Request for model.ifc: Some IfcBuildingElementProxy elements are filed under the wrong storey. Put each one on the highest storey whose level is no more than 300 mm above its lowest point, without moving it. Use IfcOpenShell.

First a look at what the model holds.

```python
import ifcopenshell
import ifcopenshell.util.element
import ifcopenshell.util.placement

model = ifcopenshell.open("model.ifc")
print(model.schema)
for storey in model.by_type("IfcBuildingStorey"):
    level = ifcopenshell.util.placement.get_storey_elevation(storey)
    count = sum(e.is_a("IfcBuildingElementProxy") for e in ifcopenshell.util.element.get_contained(storey))
    print(storey.id(), storey.Name, round(level, 3), count, sep=" | ")
```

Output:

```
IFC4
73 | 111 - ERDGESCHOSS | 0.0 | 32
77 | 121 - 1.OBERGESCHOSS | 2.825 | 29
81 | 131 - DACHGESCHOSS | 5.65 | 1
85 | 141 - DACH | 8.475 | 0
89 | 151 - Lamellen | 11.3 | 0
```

```python
import ifcopenshell
import ifcopenshell.api.spatial
import ifcopenshell.geom
import ifcopenshell.util.element
import ifcopenshell.util.placement
import ifcopenshell.util.shape
import ifcopenshell.util.unit

model = ifcopenshell.open("model.ifc")
unit_scale = ifcopenshell.util.unit.calculate_unit_scale(model)
settings = ifcopenshell.geom.settings()

levels = sorted(
    ((ifcopenshell.util.placement.get_storey_elevation(s) * unit_scale, s) for s in model.by_type("IfcBuildingStorey")),
    key=lambda pair: pair[0],
)

for e in model.by_type("IfcBuildingElementProxy"):
    current = e.ContainedInStructure[0].RelatingStructure if e.ContainedInStructure else None
    if current is None or not current.is_a("IfcBuildingStorey"):
        continue
    shape = ifcopenshell.geom.create_shape(settings, e)
    bottom = ifcopenshell.util.shape.get_shape_bottom_elevation(shape, shape.geometry)
    below = [s for level, s in levels if level <= bottom + 0.3]
    storey = below[-1] if below else levels[0][1]
    if storey != current:
        # assign_container keeps the world position.
        ifcopenshell.api.spatial.assign_container(model, products=[e], relating_structure=storey)
        print(e.id(), current.Name, "->", storey.Name)

model.write("model_rev.ifc")
```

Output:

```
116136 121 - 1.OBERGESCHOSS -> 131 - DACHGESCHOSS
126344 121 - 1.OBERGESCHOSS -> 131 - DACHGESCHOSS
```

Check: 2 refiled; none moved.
